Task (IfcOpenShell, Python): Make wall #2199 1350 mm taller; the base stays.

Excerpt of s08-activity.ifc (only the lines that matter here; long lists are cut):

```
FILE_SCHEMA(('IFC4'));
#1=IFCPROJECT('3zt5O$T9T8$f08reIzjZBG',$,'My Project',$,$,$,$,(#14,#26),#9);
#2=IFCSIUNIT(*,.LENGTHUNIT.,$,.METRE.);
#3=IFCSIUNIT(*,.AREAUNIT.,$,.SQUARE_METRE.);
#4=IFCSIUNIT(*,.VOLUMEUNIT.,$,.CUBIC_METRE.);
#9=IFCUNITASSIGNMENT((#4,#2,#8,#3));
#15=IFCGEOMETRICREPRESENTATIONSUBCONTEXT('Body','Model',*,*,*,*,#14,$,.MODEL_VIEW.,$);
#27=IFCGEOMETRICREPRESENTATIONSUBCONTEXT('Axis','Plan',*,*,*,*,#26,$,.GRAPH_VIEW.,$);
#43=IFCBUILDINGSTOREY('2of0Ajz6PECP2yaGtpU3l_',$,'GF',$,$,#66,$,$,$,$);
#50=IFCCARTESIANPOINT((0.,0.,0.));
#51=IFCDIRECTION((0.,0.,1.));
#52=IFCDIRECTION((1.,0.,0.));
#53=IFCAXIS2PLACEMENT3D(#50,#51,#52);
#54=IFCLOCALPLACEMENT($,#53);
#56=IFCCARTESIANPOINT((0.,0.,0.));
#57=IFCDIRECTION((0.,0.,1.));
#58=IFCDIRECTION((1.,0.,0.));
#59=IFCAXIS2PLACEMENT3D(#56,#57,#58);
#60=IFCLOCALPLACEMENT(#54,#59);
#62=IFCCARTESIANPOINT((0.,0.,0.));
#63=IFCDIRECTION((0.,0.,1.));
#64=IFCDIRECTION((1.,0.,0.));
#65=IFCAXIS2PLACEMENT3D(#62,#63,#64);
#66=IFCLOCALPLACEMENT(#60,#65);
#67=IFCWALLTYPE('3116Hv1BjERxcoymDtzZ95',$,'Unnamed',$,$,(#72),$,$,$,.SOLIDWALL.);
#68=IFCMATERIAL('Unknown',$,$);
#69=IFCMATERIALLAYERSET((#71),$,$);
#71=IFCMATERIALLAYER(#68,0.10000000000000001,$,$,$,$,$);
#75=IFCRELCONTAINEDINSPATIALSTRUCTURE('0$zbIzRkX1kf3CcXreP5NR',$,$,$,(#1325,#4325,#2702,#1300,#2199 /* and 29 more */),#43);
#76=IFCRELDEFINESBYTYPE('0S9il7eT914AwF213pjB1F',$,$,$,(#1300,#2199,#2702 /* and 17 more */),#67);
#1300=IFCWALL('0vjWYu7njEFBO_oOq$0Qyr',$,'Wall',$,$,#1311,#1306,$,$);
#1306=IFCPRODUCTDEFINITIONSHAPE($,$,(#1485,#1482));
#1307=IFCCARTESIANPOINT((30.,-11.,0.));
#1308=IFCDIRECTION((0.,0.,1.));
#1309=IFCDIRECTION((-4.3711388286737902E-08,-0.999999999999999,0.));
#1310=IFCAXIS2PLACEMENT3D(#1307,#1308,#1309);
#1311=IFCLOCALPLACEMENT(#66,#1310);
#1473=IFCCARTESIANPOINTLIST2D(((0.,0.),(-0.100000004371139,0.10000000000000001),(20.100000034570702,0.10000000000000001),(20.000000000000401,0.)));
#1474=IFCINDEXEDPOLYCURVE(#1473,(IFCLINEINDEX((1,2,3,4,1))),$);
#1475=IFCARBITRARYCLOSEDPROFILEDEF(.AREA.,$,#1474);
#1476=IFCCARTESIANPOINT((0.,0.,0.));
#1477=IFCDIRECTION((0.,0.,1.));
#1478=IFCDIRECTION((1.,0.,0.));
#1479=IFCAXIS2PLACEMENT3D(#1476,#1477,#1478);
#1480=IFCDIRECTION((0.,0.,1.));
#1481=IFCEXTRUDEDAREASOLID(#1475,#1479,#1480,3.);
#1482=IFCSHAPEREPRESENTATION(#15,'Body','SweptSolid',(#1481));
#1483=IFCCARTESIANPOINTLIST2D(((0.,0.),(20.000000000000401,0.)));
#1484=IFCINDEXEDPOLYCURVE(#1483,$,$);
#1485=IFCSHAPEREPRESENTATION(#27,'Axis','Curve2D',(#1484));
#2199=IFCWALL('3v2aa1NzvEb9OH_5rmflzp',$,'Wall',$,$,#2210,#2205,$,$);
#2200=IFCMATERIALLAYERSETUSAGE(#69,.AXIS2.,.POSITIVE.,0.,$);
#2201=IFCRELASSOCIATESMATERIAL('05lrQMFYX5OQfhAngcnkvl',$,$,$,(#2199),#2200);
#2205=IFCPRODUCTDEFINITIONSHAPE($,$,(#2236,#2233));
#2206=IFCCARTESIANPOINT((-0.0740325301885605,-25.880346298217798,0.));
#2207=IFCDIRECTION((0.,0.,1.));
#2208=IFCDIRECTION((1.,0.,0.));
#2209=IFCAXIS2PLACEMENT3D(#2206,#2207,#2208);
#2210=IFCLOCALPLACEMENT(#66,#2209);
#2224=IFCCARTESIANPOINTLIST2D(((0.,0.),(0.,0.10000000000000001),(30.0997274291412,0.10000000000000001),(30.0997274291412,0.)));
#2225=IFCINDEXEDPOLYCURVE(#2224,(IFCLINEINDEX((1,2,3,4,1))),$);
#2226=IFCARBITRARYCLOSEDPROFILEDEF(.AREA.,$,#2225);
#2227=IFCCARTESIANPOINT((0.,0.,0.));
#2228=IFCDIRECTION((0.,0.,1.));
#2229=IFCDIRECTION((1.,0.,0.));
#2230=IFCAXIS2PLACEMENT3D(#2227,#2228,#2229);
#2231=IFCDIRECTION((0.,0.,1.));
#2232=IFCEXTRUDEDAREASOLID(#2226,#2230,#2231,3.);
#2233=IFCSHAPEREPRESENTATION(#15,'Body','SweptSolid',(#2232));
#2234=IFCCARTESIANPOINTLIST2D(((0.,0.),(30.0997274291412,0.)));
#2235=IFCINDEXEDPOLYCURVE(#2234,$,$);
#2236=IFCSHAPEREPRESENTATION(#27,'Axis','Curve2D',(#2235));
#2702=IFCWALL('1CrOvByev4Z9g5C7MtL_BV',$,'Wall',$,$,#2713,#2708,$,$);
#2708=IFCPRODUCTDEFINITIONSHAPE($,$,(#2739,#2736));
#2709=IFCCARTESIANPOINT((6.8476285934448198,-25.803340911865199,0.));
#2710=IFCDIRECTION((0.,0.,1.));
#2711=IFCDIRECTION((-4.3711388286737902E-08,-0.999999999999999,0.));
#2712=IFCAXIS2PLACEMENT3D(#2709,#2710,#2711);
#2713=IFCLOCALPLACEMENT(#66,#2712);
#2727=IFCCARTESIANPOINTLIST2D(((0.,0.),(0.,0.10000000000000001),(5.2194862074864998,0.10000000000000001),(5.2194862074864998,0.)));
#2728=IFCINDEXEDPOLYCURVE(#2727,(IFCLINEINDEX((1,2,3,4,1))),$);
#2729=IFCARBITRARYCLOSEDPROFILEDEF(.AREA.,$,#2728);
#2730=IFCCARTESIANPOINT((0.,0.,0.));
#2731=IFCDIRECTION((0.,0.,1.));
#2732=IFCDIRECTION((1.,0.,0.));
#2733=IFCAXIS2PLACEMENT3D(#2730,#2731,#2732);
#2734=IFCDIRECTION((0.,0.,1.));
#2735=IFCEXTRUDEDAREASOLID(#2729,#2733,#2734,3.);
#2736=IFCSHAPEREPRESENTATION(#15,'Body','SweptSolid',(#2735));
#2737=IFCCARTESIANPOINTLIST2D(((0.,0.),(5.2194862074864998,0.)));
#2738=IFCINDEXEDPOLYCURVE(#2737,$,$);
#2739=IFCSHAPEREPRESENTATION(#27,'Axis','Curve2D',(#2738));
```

```python
import ifcopenshell
import ifcopenshell.geom
import ifcopenshell.util.representation
import ifcopenshell.util.shape
import ifcopenshell.util.unit

model = ifcopenshell.open("s08-activity.ifc")
unit_scale = ifcopenshell.util.unit.calculate_unit_scale(model)
settings = ifcopenshell.geom.settings()


def volume(element):
    """Net volume in cubic metres, openings subtracted."""
    shape = ifcopenshell.geom.create_shape(settings, element)
    return ifcopenshell.util.shape.get_volume(shape.geometry)


wall = model.by_guid("3v2aa1NzvEb9OH_5rmflzp")
before = volume(wall)

body = ifcopenshell.util.representation.get_representation(wall, "Model", "Body")
solid = body.Items[0]
old_height = solid.Depth
solid.Depth += 1.35 / unit_scale
after = volume(wall)

print(f"height {old_height:g} -> {solid.Depth:g}, volume {before:.3f} -> {after:.3f} m3")

model.write("s08-activity_rev.ifc")
```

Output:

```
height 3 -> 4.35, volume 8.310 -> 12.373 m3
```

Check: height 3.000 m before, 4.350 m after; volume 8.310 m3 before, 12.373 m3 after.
